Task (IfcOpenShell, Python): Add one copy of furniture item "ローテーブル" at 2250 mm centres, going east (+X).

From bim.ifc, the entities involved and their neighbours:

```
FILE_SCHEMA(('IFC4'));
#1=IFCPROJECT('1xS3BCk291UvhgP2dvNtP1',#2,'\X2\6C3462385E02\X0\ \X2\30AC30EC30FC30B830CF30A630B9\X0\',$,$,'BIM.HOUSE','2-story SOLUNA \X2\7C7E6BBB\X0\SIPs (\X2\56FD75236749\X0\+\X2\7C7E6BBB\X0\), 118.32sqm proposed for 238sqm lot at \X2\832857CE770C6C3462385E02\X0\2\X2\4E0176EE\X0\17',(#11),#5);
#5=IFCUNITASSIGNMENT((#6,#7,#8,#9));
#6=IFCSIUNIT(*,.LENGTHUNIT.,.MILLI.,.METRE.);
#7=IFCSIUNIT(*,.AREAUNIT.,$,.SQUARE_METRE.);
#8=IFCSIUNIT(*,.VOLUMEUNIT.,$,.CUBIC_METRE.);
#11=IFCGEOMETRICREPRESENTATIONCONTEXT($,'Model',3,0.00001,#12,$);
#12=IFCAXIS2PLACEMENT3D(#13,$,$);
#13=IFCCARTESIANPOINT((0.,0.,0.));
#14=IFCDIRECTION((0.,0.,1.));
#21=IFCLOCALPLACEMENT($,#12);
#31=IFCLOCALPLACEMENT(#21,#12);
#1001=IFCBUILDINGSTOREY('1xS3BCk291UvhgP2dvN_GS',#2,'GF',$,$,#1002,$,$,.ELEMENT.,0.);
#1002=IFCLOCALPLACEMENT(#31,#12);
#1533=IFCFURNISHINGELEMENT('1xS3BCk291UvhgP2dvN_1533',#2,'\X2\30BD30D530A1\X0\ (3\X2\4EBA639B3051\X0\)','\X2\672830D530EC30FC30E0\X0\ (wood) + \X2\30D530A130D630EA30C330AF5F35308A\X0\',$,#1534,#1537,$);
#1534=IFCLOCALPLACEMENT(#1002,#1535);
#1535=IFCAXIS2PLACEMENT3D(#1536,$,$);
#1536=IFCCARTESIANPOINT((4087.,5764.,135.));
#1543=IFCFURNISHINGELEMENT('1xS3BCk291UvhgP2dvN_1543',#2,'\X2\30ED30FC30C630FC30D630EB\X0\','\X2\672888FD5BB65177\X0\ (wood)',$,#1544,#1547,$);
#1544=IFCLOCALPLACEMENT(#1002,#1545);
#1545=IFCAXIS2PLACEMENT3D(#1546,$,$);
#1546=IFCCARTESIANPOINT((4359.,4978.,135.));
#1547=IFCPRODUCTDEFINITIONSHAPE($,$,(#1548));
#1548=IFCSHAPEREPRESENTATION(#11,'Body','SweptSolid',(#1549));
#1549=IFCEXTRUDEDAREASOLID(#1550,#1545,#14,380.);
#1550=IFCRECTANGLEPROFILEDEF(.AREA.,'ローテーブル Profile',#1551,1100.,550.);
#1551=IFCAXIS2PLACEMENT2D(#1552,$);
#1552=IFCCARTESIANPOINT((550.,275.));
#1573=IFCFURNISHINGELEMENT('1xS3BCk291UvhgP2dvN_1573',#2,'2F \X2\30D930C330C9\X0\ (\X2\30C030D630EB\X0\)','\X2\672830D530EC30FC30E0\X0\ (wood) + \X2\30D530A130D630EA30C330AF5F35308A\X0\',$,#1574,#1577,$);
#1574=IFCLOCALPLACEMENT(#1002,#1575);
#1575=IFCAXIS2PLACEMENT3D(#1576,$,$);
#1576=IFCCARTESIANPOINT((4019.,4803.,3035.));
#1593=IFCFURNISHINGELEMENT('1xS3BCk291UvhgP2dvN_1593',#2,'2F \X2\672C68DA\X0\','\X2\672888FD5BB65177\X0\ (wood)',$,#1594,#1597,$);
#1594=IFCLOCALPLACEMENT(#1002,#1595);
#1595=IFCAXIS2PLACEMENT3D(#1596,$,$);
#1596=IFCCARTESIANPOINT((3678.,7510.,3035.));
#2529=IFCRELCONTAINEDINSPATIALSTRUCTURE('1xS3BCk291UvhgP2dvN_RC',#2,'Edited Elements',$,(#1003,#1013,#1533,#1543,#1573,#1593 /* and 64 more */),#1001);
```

```python
import numpy as np
import ifcopenshell
import ifcopenshell.api.geometry
import ifcopenshell.api.root
import ifcopenshell.util.element
import ifcopenshell.util.placement

model = ifcopenshell.open("bim.ifc")


def reuse_history(source, copy):
    """copy_class also copies each property set's owner history, people and application; keep the originals."""
    for rel in copy.IsDefinedBy:
        if rel.is_a("IfcRelDefinesByProperties") and (history := rel.RelatingPropertyDefinition.OwnerHistory):
            rel.RelatingPropertyDefinition.OwnerHistory = source.OwnerHistory
            ifcopenshell.util.element.remove_deep2(model, history)


source = model.by_id(1543)
base = ifcopenshell.util.placement.get_local_placement(source.ObjectPlacement)
step = np.array([1.0, 0.0, 0.0]) * 2250.0

for i in range(1, 2):
    copy = ifcopenshell.api.root.copy_class(model, product=source)
    copy.Representation = ifcopenshell.util.element.copy_deep(
        model, source.Representation, exclude=["IfcGeometricRepresentationContext", "IfcRepresentationMap"]
    )
    reuse_history(source, copy)
    matrix = base.copy()
    matrix[:3, 3] += i * step
    print("added at", matrix[:3, 3].round(3) + 0.0)
    ifcopenshell.api.geometry.edit_object_placement(model, product=copy, matrix=matrix, is_si=False)

model.write("bim_updated.ifc")
```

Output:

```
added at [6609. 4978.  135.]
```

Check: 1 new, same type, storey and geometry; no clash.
